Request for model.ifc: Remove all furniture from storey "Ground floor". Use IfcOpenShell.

First a look at what the model holds.

```python
import ifcopenshell
import ifcopenshell.util.element

model = ifcopenshell.open("model.ifc")
print(model.schema)
storey = next(s for s in model.by_type("IfcBuildingStorey") if s.Name == "Ground floor")
furniture = [e for e in ifcopenshell.util.element.get_decomposition(storey) if e.is_a("IfcFurnishingElement")]
seen = {}
for e in furniture:
    element_type = ifcopenshell.util.element.get_type(e)
    name = element_type.Name if element_type not in (None, e) else None
    seen[name] = seen.get(name, 0) + 1
for name, count in sorted(seen.items(), key=str):
    print(count, "x", name)
```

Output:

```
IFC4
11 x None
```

```python
import ifcopenshell
import ifcopenshell.api.root
import ifcopenshell.util.element

model = ifcopenshell.open("model.ifc")

storey = next(s for s in model.by_type("IfcBuildingStorey") if s.Name == "Ground floor")
furniture = [e for e in ifcopenshell.util.element.get_decomposition(storey) if e.is_a("IfcFurnishingElement")]

for e in furniture:
    ifcopenshell.api.root.remove_product(model, product=e)
print(len(furniture), "removed")

model.write("model_rev.ifc")
```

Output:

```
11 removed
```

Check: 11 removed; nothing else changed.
